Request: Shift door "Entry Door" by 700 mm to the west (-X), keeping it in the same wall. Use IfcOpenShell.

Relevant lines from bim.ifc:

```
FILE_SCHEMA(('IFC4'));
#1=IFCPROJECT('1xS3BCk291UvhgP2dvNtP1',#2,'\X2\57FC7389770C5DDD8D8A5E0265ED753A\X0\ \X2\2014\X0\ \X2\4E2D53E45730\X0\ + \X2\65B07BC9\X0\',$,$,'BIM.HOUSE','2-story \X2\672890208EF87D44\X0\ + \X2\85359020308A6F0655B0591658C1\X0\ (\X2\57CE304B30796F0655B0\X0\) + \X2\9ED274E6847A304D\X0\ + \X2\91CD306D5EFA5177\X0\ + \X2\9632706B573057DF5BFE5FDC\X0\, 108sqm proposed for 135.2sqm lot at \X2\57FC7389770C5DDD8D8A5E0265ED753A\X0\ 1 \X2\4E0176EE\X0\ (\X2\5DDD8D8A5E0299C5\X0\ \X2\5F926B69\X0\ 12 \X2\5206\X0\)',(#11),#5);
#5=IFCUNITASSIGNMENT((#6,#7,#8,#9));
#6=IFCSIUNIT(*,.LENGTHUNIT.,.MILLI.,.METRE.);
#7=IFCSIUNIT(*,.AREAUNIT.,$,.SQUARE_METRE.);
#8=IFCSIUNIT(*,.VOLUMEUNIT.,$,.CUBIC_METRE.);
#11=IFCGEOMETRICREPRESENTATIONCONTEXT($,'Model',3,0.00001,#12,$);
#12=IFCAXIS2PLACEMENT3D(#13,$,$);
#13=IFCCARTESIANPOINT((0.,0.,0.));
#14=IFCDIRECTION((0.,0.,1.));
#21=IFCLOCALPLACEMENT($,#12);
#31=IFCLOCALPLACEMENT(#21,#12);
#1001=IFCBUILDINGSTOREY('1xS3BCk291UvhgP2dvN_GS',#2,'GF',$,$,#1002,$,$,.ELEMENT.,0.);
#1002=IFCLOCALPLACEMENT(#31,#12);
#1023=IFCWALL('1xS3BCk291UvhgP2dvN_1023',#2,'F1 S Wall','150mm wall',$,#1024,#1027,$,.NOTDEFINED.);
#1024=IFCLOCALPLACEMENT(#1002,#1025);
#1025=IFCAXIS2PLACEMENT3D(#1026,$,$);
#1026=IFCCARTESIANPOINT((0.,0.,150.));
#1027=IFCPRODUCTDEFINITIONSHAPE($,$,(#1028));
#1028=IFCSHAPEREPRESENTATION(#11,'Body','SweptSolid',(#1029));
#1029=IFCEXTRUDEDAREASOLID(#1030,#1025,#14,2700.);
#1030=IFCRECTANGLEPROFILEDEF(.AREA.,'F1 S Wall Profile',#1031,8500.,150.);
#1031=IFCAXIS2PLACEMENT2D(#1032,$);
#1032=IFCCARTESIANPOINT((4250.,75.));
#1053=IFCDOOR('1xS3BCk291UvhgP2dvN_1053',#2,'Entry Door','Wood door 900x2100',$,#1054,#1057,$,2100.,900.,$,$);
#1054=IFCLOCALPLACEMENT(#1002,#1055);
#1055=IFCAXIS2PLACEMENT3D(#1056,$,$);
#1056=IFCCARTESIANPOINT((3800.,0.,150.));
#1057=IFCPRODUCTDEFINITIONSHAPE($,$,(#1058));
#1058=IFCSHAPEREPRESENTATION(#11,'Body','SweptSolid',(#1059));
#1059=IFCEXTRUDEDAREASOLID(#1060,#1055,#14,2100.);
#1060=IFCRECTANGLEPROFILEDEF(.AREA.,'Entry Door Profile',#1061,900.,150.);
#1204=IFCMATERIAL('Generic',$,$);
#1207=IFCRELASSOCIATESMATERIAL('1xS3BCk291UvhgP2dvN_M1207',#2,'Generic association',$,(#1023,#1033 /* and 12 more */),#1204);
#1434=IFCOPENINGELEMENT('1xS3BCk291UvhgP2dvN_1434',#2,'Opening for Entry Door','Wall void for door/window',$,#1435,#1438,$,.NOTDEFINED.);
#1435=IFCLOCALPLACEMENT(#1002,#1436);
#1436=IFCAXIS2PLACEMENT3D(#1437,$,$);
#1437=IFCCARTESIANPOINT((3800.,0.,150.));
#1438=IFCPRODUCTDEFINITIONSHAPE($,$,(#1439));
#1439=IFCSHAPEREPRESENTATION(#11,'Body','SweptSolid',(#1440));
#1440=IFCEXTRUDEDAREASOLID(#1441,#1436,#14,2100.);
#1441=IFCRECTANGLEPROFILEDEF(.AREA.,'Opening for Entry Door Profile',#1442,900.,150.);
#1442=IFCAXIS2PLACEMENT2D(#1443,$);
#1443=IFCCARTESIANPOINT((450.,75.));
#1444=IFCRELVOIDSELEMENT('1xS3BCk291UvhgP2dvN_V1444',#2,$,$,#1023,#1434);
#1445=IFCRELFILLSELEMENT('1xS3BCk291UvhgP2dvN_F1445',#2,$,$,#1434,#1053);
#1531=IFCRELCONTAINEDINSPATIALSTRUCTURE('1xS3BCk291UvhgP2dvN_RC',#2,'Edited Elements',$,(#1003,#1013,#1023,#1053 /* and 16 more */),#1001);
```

```python
import ifcopenshell
import ifcopenshell.api.geometry
import ifcopenshell.util.placement

model = ifcopenshell.open("bim.ifc")

door = model.by_id(1053)
opening = door.FillsVoids[0].RelatingOpeningElement
wall = opening.VoidsElements[0].RelatingBuildingElement

wall_matrix = ifcopenshell.util.placement.get_local_placement(wall.ObjectPlacement)
shift = wall_matrix[:3, 0] * -700.0
before = ifcopenshell.util.placement.get_local_placement(door.ObjectPlacement)[:3, 3].copy()

# The door is not placed relative to its opening, so move both.
for product in (opening, door):
    matrix = ifcopenshell.util.placement.get_local_placement(product.ObjectPlacement)
    matrix[:3, 3] += shift
    ifcopenshell.api.geometry.edit_object_placement(model, product=product, matrix=matrix, is_si=False)

after = ifcopenshell.util.placement.get_local_placement(door.ObjectPlacement)[:3, 3]
print("door moved by", (after - before).round(3) + 0.0)

model.write("bim_updated.ifc")
```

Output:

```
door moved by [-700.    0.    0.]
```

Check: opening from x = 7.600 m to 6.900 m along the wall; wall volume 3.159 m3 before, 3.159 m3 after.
